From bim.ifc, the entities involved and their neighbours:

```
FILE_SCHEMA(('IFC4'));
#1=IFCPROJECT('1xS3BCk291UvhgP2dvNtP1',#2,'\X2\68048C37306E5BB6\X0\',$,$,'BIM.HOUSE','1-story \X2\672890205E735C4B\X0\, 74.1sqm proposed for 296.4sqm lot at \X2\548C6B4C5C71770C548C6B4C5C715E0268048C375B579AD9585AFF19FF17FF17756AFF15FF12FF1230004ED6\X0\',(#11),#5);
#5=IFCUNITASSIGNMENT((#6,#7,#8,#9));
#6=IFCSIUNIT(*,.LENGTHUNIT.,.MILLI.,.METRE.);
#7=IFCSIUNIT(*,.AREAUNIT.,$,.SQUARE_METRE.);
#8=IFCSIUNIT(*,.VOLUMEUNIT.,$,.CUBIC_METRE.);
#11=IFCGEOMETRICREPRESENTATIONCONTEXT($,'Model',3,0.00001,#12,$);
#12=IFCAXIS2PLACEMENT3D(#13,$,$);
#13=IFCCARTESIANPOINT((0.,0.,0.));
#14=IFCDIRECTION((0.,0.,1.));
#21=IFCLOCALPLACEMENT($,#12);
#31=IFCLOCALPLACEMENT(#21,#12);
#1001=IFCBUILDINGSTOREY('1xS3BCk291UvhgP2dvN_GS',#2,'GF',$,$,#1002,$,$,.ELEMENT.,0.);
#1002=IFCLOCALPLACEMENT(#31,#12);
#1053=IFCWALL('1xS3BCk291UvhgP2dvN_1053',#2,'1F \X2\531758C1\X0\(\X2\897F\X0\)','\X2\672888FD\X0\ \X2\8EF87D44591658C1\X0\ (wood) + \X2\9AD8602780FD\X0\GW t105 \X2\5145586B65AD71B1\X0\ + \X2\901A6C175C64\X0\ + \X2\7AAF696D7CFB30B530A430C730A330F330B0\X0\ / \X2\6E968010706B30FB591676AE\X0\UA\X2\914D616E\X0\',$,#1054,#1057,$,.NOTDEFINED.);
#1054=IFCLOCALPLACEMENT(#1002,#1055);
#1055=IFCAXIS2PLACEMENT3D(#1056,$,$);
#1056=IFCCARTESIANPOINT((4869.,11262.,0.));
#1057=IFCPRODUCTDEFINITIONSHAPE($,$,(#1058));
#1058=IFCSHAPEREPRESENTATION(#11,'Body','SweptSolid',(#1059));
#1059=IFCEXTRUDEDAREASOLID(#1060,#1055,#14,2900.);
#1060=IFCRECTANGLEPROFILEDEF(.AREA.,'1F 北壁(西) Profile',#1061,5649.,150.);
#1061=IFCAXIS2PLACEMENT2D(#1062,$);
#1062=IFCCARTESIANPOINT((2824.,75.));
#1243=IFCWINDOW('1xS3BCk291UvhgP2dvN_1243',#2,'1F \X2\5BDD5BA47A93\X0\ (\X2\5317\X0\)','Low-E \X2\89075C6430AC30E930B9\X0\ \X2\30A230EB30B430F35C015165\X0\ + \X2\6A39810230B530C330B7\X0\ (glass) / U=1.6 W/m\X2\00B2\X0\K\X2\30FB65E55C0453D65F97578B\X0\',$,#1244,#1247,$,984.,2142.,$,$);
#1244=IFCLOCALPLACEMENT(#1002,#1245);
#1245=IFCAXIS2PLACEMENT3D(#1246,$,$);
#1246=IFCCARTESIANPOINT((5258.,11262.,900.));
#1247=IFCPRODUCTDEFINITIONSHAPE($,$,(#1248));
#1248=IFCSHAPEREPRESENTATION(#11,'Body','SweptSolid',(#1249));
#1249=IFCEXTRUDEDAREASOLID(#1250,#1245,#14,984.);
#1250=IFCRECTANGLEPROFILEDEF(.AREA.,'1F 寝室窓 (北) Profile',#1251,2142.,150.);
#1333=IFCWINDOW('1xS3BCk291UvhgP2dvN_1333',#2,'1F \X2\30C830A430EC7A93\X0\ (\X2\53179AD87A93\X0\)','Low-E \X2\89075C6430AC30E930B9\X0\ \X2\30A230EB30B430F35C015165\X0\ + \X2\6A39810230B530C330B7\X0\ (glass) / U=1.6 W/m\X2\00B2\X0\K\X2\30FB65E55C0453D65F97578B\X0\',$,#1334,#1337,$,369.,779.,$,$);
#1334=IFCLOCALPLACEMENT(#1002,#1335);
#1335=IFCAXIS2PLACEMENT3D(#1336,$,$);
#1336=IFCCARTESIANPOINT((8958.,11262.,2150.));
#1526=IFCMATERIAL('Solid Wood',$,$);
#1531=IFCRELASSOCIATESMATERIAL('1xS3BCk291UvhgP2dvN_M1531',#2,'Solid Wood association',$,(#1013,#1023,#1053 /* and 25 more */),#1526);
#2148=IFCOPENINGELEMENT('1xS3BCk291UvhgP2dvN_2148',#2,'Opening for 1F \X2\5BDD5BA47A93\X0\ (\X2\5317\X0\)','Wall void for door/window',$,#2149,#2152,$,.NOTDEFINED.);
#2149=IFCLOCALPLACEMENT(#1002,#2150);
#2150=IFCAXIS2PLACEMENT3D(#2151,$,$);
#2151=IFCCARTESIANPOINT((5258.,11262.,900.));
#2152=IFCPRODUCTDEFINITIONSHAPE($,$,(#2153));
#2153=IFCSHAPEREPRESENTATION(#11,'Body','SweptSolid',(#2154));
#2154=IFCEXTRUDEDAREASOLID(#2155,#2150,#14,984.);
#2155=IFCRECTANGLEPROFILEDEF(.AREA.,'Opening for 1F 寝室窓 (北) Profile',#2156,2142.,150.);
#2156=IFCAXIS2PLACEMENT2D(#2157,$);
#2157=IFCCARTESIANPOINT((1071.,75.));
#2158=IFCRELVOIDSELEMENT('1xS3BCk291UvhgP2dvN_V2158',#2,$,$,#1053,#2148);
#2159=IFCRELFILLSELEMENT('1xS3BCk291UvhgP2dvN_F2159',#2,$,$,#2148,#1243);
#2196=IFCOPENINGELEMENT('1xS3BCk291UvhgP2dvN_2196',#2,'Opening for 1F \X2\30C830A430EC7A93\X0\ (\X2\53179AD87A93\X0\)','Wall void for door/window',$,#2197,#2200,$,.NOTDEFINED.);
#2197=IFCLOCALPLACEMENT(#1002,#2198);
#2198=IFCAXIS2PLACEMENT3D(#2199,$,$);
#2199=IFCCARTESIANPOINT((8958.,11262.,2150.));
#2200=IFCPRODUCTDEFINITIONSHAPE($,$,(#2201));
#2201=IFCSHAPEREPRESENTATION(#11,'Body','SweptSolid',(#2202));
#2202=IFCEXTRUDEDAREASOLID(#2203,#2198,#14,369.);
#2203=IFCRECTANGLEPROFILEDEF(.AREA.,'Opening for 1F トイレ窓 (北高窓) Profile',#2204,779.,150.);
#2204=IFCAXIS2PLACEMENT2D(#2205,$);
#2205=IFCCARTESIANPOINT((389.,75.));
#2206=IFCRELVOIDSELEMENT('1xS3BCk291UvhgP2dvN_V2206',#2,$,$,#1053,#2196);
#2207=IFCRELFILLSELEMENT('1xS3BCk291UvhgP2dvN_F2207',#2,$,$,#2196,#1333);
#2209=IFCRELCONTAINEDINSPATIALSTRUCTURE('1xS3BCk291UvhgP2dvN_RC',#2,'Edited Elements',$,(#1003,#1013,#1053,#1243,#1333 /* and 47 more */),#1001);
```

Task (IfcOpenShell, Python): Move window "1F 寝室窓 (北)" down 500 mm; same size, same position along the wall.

```python
import numpy as np
import ifcopenshell
import ifcopenshell.api.geometry
import ifcopenshell.util.placement
import ifcopenshell.util.unit

model = ifcopenshell.open("bim.ifc")
unit_scale = ifcopenshell.util.unit.calculate_unit_scale(model)

window = model.by_id(1243)
opening = window.FillsVoids[0].RelatingOpeningElement
dz = -500.0

shift = np.array([0.0, 0.0, dz])
# The window is not placed relative to its opening, so move both.
for product in (opening, window):
    matrix = ifcopenshell.util.placement.get_local_placement(product.ObjectPlacement)
    matrix[:3, 3] += shift
    ifcopenshell.api.geometry.edit_object_placement(model, product=product, matrix=matrix, is_si=False)

print(f"moved by {dz * unit_scale:+.3f} m")

model.write("bim_edited.ifc")
```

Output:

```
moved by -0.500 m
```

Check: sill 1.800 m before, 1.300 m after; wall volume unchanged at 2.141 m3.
